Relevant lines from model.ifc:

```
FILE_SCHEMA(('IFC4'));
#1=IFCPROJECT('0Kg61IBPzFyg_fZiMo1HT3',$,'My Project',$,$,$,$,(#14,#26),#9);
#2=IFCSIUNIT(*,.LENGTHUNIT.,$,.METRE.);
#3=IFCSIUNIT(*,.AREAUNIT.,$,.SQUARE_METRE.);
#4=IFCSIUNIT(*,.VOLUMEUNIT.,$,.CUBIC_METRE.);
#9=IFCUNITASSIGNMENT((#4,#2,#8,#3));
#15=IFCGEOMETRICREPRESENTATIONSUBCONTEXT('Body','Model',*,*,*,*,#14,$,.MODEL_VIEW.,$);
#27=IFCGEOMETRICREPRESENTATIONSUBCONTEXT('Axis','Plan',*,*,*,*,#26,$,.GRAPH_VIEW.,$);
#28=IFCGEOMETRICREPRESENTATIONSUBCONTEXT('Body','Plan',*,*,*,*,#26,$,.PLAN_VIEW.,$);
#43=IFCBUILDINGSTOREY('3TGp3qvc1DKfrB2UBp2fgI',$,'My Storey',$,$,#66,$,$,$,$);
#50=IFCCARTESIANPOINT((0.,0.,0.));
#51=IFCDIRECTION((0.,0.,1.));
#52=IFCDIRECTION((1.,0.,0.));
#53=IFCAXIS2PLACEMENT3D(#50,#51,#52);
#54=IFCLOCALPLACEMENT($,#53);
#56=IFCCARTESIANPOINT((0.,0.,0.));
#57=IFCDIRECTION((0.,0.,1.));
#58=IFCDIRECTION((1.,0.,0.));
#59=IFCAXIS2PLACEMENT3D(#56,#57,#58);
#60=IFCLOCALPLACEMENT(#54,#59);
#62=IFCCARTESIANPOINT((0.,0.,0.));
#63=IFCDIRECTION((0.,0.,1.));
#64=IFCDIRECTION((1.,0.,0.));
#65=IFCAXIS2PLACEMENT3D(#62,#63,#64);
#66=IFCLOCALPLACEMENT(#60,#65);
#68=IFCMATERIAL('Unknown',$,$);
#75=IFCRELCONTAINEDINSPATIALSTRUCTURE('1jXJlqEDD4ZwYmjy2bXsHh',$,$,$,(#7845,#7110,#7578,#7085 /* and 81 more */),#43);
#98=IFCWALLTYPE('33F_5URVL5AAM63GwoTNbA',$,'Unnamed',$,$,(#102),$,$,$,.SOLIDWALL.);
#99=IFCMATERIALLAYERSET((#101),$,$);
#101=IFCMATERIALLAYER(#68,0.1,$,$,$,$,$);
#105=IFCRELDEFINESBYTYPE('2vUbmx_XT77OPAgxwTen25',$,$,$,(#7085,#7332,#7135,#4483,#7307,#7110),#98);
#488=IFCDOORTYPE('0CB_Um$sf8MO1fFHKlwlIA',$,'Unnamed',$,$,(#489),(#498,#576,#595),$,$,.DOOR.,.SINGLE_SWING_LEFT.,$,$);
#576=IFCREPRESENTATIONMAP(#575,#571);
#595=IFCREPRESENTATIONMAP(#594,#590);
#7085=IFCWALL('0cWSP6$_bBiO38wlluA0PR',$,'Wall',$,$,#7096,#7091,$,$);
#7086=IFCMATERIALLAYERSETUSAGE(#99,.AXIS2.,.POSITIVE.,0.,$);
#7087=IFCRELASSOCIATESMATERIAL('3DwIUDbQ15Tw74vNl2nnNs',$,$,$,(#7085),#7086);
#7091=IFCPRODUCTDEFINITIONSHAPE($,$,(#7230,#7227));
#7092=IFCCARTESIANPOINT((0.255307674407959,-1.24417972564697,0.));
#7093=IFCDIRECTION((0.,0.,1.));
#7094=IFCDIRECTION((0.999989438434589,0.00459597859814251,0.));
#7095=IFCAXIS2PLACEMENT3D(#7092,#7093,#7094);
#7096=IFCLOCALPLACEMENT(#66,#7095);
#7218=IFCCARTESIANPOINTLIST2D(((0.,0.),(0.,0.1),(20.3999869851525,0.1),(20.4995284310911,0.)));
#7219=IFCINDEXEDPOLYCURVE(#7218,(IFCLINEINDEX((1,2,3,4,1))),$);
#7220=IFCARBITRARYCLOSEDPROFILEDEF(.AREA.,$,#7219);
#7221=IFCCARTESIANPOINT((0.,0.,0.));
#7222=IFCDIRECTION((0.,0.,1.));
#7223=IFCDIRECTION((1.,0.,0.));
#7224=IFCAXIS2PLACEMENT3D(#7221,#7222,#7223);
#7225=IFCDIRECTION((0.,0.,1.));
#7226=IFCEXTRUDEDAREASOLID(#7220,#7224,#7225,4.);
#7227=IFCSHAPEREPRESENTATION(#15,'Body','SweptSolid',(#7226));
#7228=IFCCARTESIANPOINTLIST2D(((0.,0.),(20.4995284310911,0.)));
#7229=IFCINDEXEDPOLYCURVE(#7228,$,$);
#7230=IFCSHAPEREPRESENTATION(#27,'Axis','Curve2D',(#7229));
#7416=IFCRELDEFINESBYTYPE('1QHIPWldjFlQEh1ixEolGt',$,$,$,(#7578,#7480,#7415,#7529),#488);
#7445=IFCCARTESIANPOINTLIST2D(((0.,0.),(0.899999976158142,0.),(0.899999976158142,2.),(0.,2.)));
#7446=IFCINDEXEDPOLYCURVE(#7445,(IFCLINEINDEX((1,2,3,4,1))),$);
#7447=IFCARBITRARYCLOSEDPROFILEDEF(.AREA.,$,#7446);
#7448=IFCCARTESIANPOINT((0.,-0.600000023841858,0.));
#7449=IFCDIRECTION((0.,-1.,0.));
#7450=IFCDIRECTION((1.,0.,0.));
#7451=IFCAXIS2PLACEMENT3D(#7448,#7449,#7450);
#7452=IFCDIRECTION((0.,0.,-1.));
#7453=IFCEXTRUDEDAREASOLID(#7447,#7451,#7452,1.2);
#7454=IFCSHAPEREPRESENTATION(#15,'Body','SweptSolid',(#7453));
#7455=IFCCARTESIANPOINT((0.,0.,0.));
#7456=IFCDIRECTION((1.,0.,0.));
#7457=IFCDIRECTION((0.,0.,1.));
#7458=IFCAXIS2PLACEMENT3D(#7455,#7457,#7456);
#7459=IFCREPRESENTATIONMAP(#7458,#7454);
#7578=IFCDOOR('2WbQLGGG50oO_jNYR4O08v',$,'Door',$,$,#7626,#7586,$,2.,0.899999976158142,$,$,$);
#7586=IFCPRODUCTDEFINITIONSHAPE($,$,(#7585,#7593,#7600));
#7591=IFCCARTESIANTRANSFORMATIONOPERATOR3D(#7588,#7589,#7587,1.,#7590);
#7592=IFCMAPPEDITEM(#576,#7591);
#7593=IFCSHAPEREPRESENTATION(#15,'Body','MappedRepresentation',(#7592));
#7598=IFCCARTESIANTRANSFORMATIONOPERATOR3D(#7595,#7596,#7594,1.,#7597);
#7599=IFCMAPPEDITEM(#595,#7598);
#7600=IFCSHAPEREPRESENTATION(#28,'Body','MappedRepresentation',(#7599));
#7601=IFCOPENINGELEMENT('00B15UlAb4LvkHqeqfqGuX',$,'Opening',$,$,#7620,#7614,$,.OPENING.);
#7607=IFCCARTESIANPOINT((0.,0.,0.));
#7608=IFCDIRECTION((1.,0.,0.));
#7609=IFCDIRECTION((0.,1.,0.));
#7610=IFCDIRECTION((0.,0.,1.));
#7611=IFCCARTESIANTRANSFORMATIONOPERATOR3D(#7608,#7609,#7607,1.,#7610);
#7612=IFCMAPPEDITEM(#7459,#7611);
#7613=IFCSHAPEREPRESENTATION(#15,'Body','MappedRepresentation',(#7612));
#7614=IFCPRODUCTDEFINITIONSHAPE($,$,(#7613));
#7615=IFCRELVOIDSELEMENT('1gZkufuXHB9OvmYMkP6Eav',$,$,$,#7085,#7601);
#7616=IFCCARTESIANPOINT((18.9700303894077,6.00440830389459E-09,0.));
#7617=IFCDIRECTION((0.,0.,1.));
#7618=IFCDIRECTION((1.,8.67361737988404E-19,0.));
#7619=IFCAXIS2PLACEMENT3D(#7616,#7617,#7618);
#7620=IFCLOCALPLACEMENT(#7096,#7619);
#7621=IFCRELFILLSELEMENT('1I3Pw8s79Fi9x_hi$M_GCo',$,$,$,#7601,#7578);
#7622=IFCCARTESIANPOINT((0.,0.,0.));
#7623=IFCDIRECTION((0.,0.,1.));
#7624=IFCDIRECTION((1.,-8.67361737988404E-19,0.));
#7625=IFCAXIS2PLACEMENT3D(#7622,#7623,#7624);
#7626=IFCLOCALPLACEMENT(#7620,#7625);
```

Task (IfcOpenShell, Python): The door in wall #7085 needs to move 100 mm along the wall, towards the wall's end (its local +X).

```python
import ifcopenshell
import ifcopenshell.api.geometry
import ifcopenshell.util.placement
import ifcopenshell.util.unit

model = ifcopenshell.open("model.ifc")
unit_scale = ifcopenshell.util.unit.calculate_unit_scale(model)

door = model.by_guid("2WbQLGGG50oO_jNYR4O08v")
opening = door.FillsVoids[0].RelatingOpeningElement
wall = opening.VoidsElements[0].RelatingBuildingElement

wall_matrix = ifcopenshell.util.placement.get_local_placement(wall.ObjectPlacement)
shift = wall_matrix[:3, 0] * 0.1 / unit_scale
before = ifcopenshell.util.placement.get_local_placement(door.ObjectPlacement)[:3, 3].copy()

# The door is placed relative to its opening, so it follows when the opening moves.
matrix = ifcopenshell.util.placement.get_local_placement(opening.ObjectPlacement)
matrix[:3, 3] += shift
ifcopenshell.api.geometry.edit_object_placement(
    model, product=opening, matrix=matrix, is_si=False, should_transform_children=True
)

after = ifcopenshell.util.placement.get_local_placement(door.ObjectPlacement)[:3, 3]
print("door moved by", (after - before).round(3) + 0.0)

model.write("model_updated.ifc")
```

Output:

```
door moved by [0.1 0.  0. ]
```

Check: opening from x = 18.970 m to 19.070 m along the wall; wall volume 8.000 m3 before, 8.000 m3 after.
